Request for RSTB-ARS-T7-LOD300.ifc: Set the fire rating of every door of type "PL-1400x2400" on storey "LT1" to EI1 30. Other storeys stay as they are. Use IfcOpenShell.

First a look at what the model holds.

```python
import ifcopenshell
import ifcopenshell.util.element

model = ifcopenshell.open("RSTB-ARS-T7-LOD300.ifc")
print(model.schema)
storey = next(s for s in model.by_type("IfcBuildingStorey") if s.Name == "LT1")
doors = [e for e in ifcopenshell.util.element.get_decomposition(storey) if e.is_a("IfcDoor")]
seen = {}
for e in doors:
    element_type = ifcopenshell.util.element.get_type(e)
    key = (element_type.Name if element_type != e and element_type else None, ifcopenshell.util.element.get_pset(e, "Pset_DoorCommon", "FireRating"))
    seen[key] = seen.get(key, 0) + 1
for (name, value), count in sorted(seen.items(), key=str):
    print(count, "x", name, "|", value)
```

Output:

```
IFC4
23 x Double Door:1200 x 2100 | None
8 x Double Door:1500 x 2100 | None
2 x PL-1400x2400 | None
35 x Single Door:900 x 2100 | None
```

```python
import ifcopenshell
import ifcopenshell.api.pset
import ifcopenshell.util.element

model = ifcopenshell.open("RSTB-ARS-T7-LOD300.ifc")

storey = next(s for s in model.by_type("IfcBuildingStorey") if s.Name == "LT1")
doors = [e for e in ifcopenshell.util.element.get_decomposition(storey) if e.is_a("IfcDoor")]

count = 0
for e in doors:
    element_type = ifcopenshell.util.element.get_type(e)
    if element_type in (None, e) or element_type.Name != "PL-1400x2400":
        continue
    # add_pset returns the element's existing set when there is one.
    pset = ifcopenshell.api.pset.add_pset(model, product=e, name="Pset_DoorCommon")
    ifcopenshell.api.pset.edit_pset(model, pset=pset, properties={"FireRating": "EI1 30"})
    count += 1

print(count, "doors updated")

model.write("RSTB-ARS-T7-LOD300_updated.ifc")
```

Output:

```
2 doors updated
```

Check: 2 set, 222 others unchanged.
